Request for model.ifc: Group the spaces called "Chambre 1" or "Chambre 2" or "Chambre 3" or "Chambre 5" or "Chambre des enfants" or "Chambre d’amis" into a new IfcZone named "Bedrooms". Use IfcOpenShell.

First a look at what the model holds.

```python
import ifcopenshell

model = ifcopenshell.open("model.ifc")
print(model.schema)
seen = {}
for space in model.by_type("IfcSpace"):
    seen[space.LongName] = seen.get(space.LongName, 0) + 1
for name, count in sorted(seen.items(), key=str):
    print(count, "x", name)
print("zones:", [z.Name for z in model.by_type("IfcZone")][:20])
```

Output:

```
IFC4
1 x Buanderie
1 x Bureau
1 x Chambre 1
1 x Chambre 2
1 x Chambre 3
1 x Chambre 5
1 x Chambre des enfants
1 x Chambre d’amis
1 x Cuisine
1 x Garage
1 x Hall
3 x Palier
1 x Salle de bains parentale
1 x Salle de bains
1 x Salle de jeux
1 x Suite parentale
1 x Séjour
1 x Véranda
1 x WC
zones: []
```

```python
import ifcopenshell
import ifcopenshell.api.group
import ifcopenshell.api.root

model = ifcopenshell.open("model.ifc")

names = {"Chambre 1", "Chambre 2", "Chambre 3", "Chambre 5", "Chambre des enfants", "Chambre d’amis"}
spaces = [s for s in model.by_type("IfcSpace") if s.LongName in names]

zone = ifcopenshell.api.root.create_entity(model, ifc_class="IfcZone", name="Bedrooms")
ifcopenshell.api.group.assign_group(model, products=spaces, group=zone)
print(len(spaces), "spaces in", zone.Name)

model.write("model_updated.ifc")
```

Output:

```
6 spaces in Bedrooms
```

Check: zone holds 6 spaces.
